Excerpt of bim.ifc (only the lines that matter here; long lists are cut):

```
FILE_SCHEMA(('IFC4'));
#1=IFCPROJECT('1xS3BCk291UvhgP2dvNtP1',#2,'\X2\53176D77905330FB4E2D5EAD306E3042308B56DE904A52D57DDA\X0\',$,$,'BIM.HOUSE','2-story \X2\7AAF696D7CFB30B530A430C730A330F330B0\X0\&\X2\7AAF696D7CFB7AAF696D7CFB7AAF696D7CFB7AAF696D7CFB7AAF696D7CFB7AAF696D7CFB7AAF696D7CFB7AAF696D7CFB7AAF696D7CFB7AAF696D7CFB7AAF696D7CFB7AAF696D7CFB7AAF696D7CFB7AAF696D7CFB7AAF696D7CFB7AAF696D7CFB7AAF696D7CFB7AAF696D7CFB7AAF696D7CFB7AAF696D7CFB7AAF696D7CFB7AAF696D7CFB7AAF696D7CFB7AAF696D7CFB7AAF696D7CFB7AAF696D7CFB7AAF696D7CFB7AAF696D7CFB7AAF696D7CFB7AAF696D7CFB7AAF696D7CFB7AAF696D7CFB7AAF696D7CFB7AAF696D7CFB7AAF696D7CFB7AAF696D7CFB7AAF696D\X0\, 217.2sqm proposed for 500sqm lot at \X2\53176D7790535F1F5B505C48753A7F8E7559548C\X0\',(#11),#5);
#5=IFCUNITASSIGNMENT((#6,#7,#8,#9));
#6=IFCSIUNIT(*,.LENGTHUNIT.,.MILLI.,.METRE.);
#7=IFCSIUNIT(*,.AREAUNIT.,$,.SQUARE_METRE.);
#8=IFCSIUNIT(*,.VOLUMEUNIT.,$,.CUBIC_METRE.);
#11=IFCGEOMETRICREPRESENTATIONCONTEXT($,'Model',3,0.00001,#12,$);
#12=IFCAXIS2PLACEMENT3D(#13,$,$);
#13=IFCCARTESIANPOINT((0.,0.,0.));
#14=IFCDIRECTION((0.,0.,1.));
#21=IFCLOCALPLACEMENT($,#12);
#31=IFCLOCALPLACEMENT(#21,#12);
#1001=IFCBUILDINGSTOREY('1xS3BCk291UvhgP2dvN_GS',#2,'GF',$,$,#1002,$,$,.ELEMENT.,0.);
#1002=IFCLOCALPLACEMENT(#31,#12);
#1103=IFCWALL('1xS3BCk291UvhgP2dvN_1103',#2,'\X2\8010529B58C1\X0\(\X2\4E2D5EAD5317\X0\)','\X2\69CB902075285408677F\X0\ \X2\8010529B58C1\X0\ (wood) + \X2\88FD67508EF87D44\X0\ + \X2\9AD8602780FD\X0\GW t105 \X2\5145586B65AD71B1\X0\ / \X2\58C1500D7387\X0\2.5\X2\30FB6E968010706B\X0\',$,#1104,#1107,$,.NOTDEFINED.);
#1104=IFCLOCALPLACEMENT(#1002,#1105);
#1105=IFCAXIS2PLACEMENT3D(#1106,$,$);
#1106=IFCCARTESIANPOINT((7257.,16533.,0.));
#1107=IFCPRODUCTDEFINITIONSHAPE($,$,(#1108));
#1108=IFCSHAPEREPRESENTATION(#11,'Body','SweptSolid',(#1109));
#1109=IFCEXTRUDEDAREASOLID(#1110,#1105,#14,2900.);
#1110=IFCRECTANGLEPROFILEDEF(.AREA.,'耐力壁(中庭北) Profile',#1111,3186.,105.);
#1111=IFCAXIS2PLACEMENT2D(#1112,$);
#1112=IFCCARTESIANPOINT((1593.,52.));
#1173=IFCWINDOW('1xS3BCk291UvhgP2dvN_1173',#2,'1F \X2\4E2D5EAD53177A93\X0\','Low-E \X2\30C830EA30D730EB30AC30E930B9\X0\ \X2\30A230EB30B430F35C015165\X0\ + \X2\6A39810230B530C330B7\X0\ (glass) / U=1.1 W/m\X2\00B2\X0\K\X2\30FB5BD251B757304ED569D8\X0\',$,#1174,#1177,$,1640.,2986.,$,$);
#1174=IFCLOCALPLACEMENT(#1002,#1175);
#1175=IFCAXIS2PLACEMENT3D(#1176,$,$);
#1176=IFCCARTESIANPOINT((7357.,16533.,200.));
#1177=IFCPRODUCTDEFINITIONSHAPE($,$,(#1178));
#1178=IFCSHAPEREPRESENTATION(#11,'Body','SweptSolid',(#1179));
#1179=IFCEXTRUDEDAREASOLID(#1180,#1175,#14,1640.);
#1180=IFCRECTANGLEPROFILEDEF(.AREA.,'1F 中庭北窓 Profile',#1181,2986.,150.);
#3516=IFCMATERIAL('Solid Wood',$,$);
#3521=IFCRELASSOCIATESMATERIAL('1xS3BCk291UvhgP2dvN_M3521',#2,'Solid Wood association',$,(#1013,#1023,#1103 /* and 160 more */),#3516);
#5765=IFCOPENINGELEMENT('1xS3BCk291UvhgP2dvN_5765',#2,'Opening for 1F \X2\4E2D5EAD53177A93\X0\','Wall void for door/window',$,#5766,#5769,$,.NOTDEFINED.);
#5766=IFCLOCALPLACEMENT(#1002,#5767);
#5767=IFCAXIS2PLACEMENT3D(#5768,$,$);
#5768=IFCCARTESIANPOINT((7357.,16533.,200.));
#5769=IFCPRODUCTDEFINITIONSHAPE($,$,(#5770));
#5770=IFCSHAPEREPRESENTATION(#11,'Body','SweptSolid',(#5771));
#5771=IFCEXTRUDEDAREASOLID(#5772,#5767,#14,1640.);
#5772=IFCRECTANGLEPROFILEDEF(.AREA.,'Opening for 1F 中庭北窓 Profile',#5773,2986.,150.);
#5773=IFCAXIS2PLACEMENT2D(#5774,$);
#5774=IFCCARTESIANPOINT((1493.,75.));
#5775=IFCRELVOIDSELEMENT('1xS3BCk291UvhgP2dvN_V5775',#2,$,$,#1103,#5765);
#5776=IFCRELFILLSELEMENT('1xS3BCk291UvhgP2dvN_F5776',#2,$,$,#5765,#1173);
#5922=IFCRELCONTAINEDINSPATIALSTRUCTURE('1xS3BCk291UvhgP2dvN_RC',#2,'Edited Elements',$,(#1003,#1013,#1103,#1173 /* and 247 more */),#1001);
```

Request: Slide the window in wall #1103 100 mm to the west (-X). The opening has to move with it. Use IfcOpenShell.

```python
import ifcopenshell
import ifcopenshell.api.geometry
import ifcopenshell.util.placement

model = ifcopenshell.open("bim.ifc")

window = model.by_guid("1xS3BCk291UvhgP2dvN_1173")
opening = window.FillsVoids[0].RelatingOpeningElement
wall = opening.VoidsElements[0].RelatingBuildingElement

wall_matrix = ifcopenshell.util.placement.get_local_placement(wall.ObjectPlacement)
shift = wall_matrix[:3, 0] * -100.0
before = ifcopenshell.util.placement.get_local_placement(window.ObjectPlacement)[:3, 3].copy()

# The window is not placed relative to its opening, so move both.
for product in (opening, window):
    matrix = ifcopenshell.util.placement.get_local_placement(product.ObjectPlacement)
    matrix[:3, 3] += shift
    ifcopenshell.api.geometry.edit_object_placement(model, product=product, matrix=matrix, is_si=False)

after = ifcopenshell.util.placement.get_local_placement(window.ObjectPlacement)[:3, 3]
print("window moved by", (after - before).round(3) + 0.0)

model.write("bim_updated.ifc")
```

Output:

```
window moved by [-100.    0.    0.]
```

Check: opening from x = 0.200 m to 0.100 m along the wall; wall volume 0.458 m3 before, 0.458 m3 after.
